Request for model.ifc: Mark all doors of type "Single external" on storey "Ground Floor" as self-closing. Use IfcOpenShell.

First a look at what the model holds.

```python
import ifcopenshell
import ifcopenshell.util.element

model = ifcopenshell.open("model.ifc")
print(model.schema)
storey = next(s for s in model.by_type("IfcBuildingStorey") if s.Name == "Ground Floor")
doors = [e for e in ifcopenshell.util.element.get_decomposition(storey) if e.is_a("IfcDoor")]
seen = {}
for e in doors:
    element_type = ifcopenshell.util.element.get_type(e)
    key = (element_type.Name if element_type != e and element_type else None, ifcopenshell.util.element.get_pset(e, "Pset_DoorCommon", "SelfClosing"))
    seen[key] = seen.get(key, 0) + 1
for (name, value), count in sorted(seen.items(), key=str):
    print(count, "x", name, "|", value)
```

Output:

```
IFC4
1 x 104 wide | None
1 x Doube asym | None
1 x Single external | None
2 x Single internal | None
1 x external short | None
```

```python
import ifcopenshell
import ifcopenshell.api.pset
import ifcopenshell.util.element

model = ifcopenshell.open("model.ifc")

storey = next(s for s in model.by_type("IfcBuildingStorey") if s.Name == "Ground Floor")
doors = [e for e in ifcopenshell.util.element.get_decomposition(storey) if e.is_a("IfcDoor")]

count = 0
for e in doors:
    element_type = ifcopenshell.util.element.get_type(e)
    if element_type in (None, e) or element_type.Name != "Single external":
        continue
    # add_pset returns the element's existing set when there is one.
    pset = ifcopenshell.api.pset.add_pset(model, product=e, name="Pset_DoorCommon")
    ifcopenshell.api.pset.edit_pset(model, pset=pset, properties={"SelfClosing": True})
    count += 1

print(count, "doors updated")

model.write("model_v2.ifc")
```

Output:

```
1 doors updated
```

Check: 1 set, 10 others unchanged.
